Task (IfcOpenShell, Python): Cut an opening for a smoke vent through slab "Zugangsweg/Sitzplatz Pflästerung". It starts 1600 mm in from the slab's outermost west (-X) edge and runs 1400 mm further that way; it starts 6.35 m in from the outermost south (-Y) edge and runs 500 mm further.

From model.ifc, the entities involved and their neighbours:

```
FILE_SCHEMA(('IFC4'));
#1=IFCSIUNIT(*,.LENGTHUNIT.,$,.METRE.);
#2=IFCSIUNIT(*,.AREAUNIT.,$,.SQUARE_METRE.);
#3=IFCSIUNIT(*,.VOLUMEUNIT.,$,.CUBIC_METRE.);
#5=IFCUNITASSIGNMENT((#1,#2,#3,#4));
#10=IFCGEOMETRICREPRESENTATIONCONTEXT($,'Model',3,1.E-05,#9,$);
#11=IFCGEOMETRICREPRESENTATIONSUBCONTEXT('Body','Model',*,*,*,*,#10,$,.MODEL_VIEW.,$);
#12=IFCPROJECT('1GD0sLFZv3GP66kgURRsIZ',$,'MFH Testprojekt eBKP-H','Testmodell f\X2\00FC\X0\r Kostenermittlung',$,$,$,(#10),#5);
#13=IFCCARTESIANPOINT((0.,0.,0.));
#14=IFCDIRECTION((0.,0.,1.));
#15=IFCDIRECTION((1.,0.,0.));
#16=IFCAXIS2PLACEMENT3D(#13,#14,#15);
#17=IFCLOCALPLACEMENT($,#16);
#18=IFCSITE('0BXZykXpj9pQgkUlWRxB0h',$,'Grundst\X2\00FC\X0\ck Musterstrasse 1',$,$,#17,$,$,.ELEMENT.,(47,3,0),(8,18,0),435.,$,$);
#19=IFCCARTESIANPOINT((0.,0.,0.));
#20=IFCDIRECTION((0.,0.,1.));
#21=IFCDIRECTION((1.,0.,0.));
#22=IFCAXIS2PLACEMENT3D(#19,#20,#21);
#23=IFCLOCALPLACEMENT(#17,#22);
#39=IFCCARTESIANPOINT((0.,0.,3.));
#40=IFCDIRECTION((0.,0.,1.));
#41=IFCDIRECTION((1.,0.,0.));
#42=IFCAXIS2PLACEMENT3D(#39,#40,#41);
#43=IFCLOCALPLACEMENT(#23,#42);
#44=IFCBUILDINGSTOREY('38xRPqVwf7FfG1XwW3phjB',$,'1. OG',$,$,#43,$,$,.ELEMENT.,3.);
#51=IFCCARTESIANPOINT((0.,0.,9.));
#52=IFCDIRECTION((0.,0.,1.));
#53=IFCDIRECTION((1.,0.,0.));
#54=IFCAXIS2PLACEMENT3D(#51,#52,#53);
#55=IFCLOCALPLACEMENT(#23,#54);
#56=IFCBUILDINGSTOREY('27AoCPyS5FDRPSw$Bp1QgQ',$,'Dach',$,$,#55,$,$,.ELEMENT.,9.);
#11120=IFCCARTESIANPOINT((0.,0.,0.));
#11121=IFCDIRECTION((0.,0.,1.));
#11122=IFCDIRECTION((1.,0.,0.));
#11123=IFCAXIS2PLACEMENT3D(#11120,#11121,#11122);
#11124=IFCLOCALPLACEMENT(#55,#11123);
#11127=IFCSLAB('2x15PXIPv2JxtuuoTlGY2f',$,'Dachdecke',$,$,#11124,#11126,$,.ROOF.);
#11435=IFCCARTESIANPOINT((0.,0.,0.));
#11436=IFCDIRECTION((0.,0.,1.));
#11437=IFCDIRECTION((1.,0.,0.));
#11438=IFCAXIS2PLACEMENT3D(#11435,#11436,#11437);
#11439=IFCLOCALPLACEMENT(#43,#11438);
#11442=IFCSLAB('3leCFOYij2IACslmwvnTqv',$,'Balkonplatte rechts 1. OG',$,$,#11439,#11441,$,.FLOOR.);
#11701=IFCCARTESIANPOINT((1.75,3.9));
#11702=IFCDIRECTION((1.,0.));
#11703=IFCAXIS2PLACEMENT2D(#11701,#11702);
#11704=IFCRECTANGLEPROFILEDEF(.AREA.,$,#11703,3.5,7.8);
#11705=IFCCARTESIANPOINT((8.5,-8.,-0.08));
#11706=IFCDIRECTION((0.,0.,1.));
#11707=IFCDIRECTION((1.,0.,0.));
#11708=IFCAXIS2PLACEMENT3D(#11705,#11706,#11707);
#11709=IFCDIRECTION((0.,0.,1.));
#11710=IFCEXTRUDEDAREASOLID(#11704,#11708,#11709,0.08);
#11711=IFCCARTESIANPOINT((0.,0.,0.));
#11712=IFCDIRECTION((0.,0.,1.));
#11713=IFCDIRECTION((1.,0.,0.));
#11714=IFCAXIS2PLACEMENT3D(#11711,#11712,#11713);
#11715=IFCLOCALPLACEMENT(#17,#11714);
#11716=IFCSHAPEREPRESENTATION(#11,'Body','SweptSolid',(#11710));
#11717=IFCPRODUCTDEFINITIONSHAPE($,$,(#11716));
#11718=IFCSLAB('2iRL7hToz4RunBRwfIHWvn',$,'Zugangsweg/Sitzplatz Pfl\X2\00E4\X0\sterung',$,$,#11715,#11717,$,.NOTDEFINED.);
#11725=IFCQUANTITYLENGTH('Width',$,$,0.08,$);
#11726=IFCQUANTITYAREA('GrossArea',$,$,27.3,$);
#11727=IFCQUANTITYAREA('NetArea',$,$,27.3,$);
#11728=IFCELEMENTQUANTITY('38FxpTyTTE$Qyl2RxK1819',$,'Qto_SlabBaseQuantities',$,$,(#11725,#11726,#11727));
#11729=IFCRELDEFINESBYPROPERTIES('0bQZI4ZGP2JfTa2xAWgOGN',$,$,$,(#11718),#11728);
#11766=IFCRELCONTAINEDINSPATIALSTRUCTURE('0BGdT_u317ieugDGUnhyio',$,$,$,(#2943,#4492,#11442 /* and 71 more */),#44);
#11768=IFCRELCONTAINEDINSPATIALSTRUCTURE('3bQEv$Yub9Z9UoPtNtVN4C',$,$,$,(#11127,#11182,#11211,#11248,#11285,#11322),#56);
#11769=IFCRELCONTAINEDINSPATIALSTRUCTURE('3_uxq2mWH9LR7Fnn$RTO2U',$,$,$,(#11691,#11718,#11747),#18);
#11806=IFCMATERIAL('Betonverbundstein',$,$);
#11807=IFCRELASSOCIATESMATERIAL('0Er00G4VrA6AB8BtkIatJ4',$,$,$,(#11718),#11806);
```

```python
import numpy as np
import ifcopenshell
import ifcopenshell.api.feature
import ifcopenshell.api.geometry
import ifcopenshell.api.pset
import ifcopenshell.api.root
import ifcopenshell.geom
import ifcopenshell.util.element
import ifcopenshell.util.placement
import ifcopenshell.util.representation
import ifcopenshell.util.shape
import ifcopenshell.util.unit

model = ifcopenshell.open("model.ifc")
unit_scale = ifcopenshell.util.unit.calculate_unit_scale(model)
area_scale = ifcopenshell.util.unit.calculate_unit_scale(model, "AREAUNIT")
settings = ifcopenshell.geom.settings()


def volume(element):
    """Net volume in cubic metres, openings subtracted."""
    shape = ifcopenshell.geom.create_shape(settings, element)
    return ifcopenshell.util.shape.get_volume(shape.geometry)


slab = model.by_guid("2iRL7hToz4RunBRwfIHWvn")
before = volume(slab)

# Extent in the slab's own axes, in metres. The edges named are its -X and -Y sides.
slab_shape = ifcopenshell.geom.create_shape(settings, slab)
vertices = ifcopenshell.util.shape.get_vertices(slab_shape.geometry)
x_min, y_min, bottom = vertices.min(axis=0)
top = vertices[:, 2].max()

opening = ifcopenshell.api.root.create_entity(model, ifc_class="IfcOpeningElement", name="Smoke vent opening", predefined_type="OPENING")
context = ifcopenshell.util.representation.get_context(model, "Model", "Body", "MODEL_VIEW")
width, depth = 1.4, 0.5
outline = [(0.0, 0.0), (width, 0.0), (width, depth), (0.0, depth), (0.0, 0.0)]
# Overshoot both faces by 50 mm so the cut is clean.
shape = ifcopenshell.api.geometry.add_slab_representation(
    model, context=context, depth=top - bottom + 0.1, polyline=outline
)
ifcopenshell.api.geometry.assign_representation(model, product=opening, representation=shape)

matrix = ifcopenshell.util.placement.get_local_placement(slab.ObjectPlacement)
matrix[:, 3] = matrix @ np.append(np.array([x_min + 1.6, y_min + 6.35, bottom - 0.05]) / unit_scale, 1.0)
ifcopenshell.api.geometry.edit_object_placement(model, product=opening, matrix=matrix, is_si=False)
ifcopenshell.api.feature.add_feature(model, feature=opening, element=slab)

after = volume(slab)

# Update the slab's stored quantities.
qto = model.by_id(ifcopenshell.util.element.get_pset(slab, "Qto_SlabBaseQuantities", should_inherit=False)["id"])
ifcopenshell.api.pset.edit_qto(model, qto=qto, properties={"NetArea": after / (top - bottom) / area_scale})

print(f"slab volume {before:.3f} -> {after:.3f} m3")

model.write("model_rev.ifc")
```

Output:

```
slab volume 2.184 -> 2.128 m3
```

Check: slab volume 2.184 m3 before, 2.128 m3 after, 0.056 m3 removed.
